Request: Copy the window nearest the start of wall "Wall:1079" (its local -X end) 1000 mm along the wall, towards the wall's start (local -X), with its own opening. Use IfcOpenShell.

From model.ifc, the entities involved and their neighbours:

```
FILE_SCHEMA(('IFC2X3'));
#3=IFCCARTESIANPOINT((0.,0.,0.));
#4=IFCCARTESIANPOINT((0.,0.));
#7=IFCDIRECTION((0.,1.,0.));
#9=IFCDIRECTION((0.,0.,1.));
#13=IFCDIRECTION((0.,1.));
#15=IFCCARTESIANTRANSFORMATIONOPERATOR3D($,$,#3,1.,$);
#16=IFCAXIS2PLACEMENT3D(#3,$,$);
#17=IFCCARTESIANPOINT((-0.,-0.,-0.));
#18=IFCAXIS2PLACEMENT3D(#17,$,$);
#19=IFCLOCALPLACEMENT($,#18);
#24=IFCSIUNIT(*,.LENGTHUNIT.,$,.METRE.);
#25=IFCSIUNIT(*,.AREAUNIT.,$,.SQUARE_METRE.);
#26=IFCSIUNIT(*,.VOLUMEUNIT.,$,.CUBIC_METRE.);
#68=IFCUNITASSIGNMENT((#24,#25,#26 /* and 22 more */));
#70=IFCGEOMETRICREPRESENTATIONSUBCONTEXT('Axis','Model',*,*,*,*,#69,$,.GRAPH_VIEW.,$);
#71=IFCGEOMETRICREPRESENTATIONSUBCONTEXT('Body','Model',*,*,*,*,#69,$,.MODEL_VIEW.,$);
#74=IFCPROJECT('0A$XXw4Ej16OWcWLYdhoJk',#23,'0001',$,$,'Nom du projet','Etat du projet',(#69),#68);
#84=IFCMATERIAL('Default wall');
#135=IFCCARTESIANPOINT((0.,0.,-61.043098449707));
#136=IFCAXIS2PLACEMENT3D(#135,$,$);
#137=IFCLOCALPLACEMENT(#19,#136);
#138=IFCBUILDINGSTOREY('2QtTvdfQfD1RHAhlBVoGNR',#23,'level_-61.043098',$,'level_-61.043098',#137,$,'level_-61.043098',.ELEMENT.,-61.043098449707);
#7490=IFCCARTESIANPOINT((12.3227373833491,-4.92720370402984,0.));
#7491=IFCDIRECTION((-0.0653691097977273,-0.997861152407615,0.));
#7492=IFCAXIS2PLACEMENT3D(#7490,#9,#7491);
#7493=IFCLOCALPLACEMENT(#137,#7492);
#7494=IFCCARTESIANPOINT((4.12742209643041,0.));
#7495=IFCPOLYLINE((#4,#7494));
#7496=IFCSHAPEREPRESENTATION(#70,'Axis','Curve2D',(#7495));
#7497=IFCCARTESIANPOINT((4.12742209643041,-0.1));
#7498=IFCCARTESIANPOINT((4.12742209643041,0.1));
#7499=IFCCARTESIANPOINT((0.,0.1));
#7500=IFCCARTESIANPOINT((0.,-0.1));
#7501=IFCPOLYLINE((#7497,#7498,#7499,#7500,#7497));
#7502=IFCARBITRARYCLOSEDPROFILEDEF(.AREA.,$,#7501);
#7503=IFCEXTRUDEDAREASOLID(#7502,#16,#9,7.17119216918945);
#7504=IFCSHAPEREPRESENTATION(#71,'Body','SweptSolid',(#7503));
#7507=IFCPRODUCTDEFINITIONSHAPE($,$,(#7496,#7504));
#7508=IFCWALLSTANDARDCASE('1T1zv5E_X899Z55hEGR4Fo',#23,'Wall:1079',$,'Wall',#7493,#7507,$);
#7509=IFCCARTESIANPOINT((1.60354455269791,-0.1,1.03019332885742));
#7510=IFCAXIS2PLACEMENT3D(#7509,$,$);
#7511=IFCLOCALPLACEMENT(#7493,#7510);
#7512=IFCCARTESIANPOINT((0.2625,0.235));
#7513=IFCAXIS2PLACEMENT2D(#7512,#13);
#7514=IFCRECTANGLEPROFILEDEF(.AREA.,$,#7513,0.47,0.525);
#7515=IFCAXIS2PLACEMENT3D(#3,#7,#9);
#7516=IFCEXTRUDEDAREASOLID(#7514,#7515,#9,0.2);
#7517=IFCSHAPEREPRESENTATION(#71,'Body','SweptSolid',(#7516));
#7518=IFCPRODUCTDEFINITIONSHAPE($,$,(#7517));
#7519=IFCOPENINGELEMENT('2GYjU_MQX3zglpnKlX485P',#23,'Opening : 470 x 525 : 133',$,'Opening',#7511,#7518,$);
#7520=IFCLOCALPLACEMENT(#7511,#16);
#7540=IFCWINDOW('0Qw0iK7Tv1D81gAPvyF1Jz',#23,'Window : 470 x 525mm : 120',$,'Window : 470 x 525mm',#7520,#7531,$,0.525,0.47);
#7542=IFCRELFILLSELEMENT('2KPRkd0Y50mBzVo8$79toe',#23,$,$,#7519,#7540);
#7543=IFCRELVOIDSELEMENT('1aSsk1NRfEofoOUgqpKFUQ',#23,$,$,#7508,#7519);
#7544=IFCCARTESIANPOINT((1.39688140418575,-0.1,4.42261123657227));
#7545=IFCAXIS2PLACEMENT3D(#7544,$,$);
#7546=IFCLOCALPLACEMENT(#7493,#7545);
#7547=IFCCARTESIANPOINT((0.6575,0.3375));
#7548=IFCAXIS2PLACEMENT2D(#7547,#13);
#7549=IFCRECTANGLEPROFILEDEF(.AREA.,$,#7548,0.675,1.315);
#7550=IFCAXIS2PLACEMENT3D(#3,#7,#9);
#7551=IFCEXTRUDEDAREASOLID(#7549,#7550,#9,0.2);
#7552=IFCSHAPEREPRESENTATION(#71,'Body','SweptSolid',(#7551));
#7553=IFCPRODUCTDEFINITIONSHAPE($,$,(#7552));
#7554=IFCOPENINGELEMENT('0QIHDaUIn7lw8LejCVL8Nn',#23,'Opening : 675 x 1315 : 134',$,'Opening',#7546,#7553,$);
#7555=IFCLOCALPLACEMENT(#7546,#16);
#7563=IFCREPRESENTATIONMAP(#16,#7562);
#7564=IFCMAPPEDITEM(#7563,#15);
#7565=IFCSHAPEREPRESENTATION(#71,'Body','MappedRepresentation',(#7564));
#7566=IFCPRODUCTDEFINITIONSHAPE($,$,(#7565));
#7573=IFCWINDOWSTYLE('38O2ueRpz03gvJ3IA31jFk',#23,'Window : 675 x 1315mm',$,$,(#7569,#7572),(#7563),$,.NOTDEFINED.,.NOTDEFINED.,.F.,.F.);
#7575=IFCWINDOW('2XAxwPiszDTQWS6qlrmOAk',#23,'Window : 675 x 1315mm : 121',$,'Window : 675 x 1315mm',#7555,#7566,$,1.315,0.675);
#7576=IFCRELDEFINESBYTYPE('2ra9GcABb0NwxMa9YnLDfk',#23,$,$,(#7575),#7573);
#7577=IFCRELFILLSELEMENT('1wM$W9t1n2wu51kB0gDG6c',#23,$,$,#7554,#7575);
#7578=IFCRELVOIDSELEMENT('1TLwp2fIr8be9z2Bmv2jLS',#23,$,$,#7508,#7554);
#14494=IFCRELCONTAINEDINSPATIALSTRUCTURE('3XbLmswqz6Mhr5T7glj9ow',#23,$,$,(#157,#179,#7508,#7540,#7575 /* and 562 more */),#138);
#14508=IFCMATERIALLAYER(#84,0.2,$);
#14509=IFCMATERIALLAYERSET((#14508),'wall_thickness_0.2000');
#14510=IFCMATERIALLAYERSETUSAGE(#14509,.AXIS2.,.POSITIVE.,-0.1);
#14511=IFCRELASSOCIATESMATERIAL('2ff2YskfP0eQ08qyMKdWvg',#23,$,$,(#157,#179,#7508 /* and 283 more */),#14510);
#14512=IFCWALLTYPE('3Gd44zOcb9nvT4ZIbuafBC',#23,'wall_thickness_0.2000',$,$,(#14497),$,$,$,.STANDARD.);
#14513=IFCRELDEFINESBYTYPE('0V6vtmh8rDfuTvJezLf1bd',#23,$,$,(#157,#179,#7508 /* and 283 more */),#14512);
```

```python
import ifcopenshell
import ifcopenshell.api.feature
import ifcopenshell.api.geometry
import ifcopenshell.api.root
import ifcopenshell.geom
import ifcopenshell.util.element
import ifcopenshell.util.placement
import ifcopenshell.util.shape

model = ifcopenshell.open("model.ifc")
settings = ifcopenshell.geom.settings()


def volume(element):
    """Net volume in cubic metres, openings subtracted."""
    shape = ifcopenshell.geom.create_shape(settings, element)
    return ifcopenshell.util.shape.get_volume(shape.geometry)


window = model.by_guid("2XAxwPiszDTQWS6qlrmOAk")
opening = window.FillsVoids[0].RelatingOpeningElement
wall = opening.VoidsElements[0].RelatingBuildingElement
before = volume(wall)
shift = ifcopenshell.util.placement.get_local_placement(wall.ObjectPlacement)[:3, 0] * -1.0

# copy_class copies the void relationship, type, container and properties, but no geometry.
new_opening = ifcopenshell.api.root.copy_class(model, product=opening)
new_opening.Representation = ifcopenshell.util.element.copy_deep(
    model, opening.Representation, exclude=["IfcGeometricRepresentationContext", "IfcRepresentationMap"]
)
new_opening.Name = "Opening : 675 x 1315"
new_window = ifcopenshell.api.root.copy_class(model, product=window)
new_window.Representation = ifcopenshell.util.element.copy_deep(
    model, window.Representation, exclude=["IfcGeometricRepresentationContext", "IfcRepresentationMap"]
)
new_window.Name = "Window : 675 x 1315mm"
fills = ifcopenshell.api.feature.add_filling(model, opening=new_opening, element=new_window)
fills.OwnerHistory = new_window.OwnerHistory  # required in IFC2X3

for old, new in ((opening, new_opening), (window, new_window)):
    matrix = ifcopenshell.util.placement.get_local_placement(old.ObjectPlacement)
    matrix[:3, 3] += shift
    ifcopenshell.api.geometry.edit_object_placement(model, product=new, matrix=matrix, is_si=False)

after = volume(wall)

print(f"wall volume {before:.3f} -> {after:.3f} m3")

model.write("model_v2.ifc")
```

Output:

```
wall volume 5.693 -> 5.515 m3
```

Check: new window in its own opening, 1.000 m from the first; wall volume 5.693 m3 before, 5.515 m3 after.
